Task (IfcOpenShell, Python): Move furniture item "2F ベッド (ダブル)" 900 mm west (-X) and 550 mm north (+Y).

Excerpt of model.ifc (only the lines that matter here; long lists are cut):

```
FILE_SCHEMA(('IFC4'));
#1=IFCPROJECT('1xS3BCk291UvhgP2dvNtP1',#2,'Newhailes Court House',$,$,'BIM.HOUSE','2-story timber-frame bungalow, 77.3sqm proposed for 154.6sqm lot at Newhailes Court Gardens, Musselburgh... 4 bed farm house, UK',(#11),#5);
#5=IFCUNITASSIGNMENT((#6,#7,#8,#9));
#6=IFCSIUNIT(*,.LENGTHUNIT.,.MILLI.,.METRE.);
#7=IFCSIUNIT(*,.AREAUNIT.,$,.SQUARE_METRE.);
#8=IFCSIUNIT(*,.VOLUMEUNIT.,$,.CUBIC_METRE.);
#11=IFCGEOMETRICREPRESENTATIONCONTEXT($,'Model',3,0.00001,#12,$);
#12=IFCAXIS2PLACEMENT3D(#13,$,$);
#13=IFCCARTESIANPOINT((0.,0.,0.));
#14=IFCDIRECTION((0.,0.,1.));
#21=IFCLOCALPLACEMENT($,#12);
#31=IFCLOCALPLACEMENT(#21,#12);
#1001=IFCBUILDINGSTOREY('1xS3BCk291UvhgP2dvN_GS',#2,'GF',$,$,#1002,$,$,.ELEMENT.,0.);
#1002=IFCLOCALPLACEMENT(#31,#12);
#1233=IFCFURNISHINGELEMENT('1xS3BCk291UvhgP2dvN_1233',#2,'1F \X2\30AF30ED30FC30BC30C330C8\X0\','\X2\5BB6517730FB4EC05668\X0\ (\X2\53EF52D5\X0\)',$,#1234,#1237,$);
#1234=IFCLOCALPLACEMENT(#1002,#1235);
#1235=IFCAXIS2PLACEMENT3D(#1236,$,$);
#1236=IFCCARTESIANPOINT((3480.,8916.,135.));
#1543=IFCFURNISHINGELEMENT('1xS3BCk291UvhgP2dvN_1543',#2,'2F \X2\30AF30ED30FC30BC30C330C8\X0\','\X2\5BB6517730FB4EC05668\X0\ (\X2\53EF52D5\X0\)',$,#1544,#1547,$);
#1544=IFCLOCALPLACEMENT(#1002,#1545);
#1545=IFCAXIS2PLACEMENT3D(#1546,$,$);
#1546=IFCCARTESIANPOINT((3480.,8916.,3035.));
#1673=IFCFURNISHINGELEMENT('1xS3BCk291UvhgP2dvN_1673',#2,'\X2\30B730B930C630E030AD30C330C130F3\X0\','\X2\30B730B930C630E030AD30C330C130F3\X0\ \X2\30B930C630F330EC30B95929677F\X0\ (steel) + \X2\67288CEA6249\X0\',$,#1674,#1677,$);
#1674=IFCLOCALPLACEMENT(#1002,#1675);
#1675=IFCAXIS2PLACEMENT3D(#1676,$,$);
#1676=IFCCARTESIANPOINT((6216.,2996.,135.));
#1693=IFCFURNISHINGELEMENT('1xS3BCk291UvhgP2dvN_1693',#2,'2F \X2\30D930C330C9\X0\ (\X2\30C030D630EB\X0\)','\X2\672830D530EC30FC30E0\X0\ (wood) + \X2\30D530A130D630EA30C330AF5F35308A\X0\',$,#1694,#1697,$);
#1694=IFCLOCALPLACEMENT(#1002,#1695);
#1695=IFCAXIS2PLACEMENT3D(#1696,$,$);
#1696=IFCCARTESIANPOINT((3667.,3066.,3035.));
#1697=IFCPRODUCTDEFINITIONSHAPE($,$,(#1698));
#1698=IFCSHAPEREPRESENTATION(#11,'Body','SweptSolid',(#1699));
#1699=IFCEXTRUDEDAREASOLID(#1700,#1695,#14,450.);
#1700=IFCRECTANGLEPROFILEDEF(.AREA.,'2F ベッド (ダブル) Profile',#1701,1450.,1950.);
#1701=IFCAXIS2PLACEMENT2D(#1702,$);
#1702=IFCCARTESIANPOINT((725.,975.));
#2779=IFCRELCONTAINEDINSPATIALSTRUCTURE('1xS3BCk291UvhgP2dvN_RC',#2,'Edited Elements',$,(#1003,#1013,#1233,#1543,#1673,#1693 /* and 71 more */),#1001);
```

```python
import ifcopenshell
import ifcopenshell.api.geometry
import ifcopenshell.util.placement

model = ifcopenshell.open("model.ifc")

item = model.by_guid("1xS3BCk291UvhgP2dvN_1693")
matrix = ifcopenshell.util.placement.get_local_placement(item.ObjectPlacement)
matrix[0, 3] -= 900.0
matrix[1, 3] += 550.0
ifcopenshell.api.geometry.edit_object_placement(model, product=item, matrix=matrix, is_si=False)

print(ifcopenshell.util.placement.get_local_placement(item.ObjectPlacement).round(3) + 0.0)

model.write("model_edited.ifc")
```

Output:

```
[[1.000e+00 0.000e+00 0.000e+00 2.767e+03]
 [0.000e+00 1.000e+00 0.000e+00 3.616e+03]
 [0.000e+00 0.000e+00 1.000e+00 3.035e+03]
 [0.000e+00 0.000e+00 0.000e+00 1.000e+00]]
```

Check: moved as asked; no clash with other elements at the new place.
